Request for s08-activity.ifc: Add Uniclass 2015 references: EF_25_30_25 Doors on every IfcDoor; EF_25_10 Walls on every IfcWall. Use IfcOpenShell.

First a look at what the model holds.

```python
import ifcopenshell

model = ifcopenshell.open("s08-activity.ifc")
print(model.schema)
print("classifications:", [c.Name for c in model.by_type("IfcClassification")])
for ifc_class in ("IfcDoor", "IfcRoof", "IfcStair", "IfcWall", "IfcWindow"):
    print(ifc_class, len(model.by_type(ifc_class)))
```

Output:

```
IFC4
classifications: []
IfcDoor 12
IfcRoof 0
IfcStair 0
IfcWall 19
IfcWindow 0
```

```python
import ifcopenshell
import ifcopenshell.api.classification

model = ifcopenshell.open("s08-activity.ifc")

system = ifcopenshell.api.classification.add_classification(model, classification="Uniclass 2015")

codes = {
    "IfcDoor": ("EF_25_30_25", "Doors"),
    "IfcWall": ("EF_25_10", "Walls"),
}
for ifc_class, (code, name) in codes.items():
    products = model.by_type(ifc_class)
    ifcopenshell.api.classification.add_reference(
        model, products=products, classification=system, identification=code, name=name
    )
    print(code, len(products))

model.write("s08-activity_v2.ifc")
```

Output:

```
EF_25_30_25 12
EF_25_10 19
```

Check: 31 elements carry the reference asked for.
